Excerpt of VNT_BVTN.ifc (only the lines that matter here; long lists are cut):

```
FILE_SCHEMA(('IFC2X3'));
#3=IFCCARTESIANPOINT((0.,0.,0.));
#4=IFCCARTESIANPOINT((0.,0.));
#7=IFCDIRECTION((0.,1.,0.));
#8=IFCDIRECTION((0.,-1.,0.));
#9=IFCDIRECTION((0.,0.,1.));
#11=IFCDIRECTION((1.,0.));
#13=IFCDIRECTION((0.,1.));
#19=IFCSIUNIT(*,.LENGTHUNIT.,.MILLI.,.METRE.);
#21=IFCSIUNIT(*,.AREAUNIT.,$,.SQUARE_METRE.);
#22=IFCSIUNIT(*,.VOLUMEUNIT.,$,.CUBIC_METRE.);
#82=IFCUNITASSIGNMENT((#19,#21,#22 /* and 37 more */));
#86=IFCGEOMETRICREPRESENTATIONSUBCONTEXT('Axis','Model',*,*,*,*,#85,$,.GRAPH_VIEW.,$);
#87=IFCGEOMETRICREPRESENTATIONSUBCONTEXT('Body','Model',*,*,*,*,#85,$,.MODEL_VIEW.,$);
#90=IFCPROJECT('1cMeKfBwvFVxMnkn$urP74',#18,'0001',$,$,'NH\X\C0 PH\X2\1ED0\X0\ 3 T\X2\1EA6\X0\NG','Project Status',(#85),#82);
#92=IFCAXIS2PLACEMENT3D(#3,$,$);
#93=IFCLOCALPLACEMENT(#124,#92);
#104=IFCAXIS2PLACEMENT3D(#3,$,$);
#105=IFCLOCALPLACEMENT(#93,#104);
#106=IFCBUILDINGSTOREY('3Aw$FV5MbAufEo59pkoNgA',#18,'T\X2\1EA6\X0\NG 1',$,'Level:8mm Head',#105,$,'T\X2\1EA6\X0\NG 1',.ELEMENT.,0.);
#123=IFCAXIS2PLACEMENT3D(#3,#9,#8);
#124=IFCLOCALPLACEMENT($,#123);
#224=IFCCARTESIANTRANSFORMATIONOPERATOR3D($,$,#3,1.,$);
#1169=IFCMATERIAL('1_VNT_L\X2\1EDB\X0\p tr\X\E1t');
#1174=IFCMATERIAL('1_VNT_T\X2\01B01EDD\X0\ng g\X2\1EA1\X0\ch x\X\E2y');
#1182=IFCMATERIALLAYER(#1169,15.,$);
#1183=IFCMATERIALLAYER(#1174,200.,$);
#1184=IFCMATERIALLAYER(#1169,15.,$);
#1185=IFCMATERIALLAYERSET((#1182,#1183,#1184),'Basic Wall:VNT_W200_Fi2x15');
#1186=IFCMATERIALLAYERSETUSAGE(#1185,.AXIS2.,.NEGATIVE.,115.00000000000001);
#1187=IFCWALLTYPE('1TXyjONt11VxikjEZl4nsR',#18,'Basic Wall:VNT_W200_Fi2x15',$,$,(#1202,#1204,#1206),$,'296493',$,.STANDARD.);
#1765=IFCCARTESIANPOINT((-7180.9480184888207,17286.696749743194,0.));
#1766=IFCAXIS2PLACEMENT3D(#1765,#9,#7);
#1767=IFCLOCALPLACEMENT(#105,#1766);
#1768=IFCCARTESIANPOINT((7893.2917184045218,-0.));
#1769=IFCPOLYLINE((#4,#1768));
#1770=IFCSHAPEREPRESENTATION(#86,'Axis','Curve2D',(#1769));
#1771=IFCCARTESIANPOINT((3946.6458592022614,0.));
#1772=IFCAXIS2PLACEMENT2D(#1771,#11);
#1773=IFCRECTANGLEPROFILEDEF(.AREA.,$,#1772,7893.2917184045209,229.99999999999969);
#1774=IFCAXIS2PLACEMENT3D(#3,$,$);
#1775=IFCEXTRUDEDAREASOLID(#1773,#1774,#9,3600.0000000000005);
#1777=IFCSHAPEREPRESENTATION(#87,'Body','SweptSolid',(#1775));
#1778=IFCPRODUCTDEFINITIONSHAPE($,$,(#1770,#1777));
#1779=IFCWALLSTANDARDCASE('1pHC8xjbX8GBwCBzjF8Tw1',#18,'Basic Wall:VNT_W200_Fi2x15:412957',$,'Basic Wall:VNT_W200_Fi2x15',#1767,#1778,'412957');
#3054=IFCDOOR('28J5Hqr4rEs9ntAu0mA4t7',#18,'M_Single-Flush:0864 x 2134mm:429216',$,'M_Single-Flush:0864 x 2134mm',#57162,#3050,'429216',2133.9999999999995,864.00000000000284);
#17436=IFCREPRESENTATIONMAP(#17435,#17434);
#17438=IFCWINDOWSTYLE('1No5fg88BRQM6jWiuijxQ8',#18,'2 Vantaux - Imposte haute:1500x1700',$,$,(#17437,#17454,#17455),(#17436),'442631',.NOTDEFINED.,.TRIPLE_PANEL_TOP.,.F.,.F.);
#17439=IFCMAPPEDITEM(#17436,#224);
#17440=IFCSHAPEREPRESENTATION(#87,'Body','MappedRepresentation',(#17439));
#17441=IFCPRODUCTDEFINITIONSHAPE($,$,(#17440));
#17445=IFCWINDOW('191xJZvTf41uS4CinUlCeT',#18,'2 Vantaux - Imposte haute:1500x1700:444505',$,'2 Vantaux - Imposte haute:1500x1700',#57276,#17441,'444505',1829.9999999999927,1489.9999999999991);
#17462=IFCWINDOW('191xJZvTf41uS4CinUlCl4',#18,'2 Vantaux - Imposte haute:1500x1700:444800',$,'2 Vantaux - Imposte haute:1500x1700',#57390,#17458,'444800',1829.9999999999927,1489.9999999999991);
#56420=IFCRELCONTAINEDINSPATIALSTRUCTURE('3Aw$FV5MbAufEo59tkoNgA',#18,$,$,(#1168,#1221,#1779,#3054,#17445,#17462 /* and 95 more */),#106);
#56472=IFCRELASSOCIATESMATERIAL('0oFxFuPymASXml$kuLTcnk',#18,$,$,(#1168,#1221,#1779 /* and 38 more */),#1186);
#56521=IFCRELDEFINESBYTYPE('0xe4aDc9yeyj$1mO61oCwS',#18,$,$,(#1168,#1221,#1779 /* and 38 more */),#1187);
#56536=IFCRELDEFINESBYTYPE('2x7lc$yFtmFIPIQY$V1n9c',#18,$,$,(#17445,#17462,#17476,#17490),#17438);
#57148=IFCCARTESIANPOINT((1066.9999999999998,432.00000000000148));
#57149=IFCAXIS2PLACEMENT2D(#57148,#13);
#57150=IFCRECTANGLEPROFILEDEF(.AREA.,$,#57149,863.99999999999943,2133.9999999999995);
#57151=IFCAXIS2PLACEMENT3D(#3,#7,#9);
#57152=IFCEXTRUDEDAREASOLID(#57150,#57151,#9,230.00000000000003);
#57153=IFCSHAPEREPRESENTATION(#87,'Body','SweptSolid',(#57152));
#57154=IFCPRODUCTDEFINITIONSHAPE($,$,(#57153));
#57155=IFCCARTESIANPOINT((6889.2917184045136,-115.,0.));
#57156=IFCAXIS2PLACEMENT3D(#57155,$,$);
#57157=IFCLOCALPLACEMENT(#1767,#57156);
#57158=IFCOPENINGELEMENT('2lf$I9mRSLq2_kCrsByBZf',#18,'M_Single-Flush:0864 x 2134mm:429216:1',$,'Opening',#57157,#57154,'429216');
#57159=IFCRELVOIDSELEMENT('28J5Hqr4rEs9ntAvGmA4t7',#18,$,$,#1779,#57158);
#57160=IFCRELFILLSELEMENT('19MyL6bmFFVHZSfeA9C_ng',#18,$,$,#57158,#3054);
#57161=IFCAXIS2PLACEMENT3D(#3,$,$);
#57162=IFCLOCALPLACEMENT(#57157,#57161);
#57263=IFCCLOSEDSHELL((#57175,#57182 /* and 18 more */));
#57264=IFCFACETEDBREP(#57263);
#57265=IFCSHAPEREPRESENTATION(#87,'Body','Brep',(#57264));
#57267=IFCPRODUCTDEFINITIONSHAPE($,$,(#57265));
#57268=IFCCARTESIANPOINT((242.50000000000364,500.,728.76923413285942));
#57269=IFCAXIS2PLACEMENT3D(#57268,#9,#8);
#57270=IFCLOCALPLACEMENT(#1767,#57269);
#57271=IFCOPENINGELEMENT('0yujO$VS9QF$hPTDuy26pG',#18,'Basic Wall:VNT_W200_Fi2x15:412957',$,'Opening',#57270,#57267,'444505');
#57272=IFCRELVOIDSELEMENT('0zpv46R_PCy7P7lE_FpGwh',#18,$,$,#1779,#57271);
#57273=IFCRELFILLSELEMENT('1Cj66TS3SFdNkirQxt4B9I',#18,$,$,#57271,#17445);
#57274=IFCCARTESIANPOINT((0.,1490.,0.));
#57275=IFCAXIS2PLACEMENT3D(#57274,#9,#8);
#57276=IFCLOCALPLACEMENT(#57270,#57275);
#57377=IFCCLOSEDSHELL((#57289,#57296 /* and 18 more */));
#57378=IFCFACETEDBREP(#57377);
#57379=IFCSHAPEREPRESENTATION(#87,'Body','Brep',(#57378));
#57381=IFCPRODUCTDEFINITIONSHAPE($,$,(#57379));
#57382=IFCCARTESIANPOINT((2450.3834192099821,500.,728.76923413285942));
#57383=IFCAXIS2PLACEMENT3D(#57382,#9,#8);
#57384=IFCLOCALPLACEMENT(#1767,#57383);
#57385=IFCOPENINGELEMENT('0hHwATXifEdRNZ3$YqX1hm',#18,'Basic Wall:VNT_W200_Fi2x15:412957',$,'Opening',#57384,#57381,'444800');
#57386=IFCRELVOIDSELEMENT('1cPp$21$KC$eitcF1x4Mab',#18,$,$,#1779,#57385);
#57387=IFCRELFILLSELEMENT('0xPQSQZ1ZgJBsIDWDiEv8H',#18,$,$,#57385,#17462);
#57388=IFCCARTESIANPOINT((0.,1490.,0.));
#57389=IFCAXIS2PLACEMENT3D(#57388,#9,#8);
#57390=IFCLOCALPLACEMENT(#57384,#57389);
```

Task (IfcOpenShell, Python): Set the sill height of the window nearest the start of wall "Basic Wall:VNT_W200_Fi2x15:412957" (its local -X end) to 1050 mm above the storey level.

```python
import numpy as np
import ifcopenshell
import ifcopenshell.api.geometry
import ifcopenshell.geom
import ifcopenshell.util.element
import ifcopenshell.util.placement
import ifcopenshell.util.shape
import ifcopenshell.util.unit

model = ifcopenshell.open("VNT_BVTN.ifc")
unit_scale = ifcopenshell.util.unit.calculate_unit_scale(model)

window = model.by_id(17445)
opening = window.FillsVoids[0].RelatingOpeningElement
storey = ifcopenshell.util.element.get_container(window, ifc_class="IfcBuildingStorey")
level = ifcopenshell.util.placement.get_local_placement(storey.ObjectPlacement)[2, 3]

# The opening's origin need not be at the sill, so measure its lowest point.
shape = ifcopenshell.geom.create_shape(ifcopenshell.geom.settings(), opening)
bottom = ifcopenshell.util.shape.get_shape_bottom_elevation(shape, shape.geometry) / unit_scale
dz = level + 1.05 / unit_scale - bottom

shift = np.array([0.0, 0.0, dz])
# The window is placed relative to its opening, so it follows when the opening moves.
matrix = ifcopenshell.util.placement.get_local_placement(opening.ObjectPlacement)
matrix[:3, 3] += shift
ifcopenshell.api.geometry.edit_object_placement(
    model, product=opening, matrix=matrix, is_si=False, should_transform_children=True
)

print(f"moved by {dz * unit_scale:+.3f} m")

model.write("VNT_BVTN_updated.ifc")
```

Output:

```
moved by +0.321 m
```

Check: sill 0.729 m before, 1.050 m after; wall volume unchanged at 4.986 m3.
